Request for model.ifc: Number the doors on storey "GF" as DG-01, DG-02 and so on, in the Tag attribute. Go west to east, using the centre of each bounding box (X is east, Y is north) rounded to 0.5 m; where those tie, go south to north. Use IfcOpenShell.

First a look at what the model holds.

```python
import ifcopenshell
import ifcopenshell.util.element
import ifcopenshell.util.placement

model = ifcopenshell.open("model.ifc")
print(model.schema)
storey = next(s for s in model.by_type("IfcBuildingStorey") if s.Name == "GF")
doors = [e for e in ifcopenshell.util.element.get_decomposition(storey) if e.is_a("IfcDoor")]
for e in sorted(doors, key=lambda e: e.id()):
    origin = ifcopenshell.util.placement.get_local_placement(e.ObjectPlacement)[:3, 3]
    print(e.id(), e.Tag, e.Name, origin.round(2) + 0.0, sep=" | ")
```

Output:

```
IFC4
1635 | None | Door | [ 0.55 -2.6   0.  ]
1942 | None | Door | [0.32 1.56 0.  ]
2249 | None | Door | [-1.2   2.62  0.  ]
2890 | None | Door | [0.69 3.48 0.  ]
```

```python
import ifcopenshell
import ifcopenshell.geom
import ifcopenshell.util.element
import ifcopenshell.util.shape

model = ifcopenshell.open("model.ifc")
settings = ifcopenshell.geom.settings()
settings.set("use-world-coords", True)


def centre(element):
    shape = ifcopenshell.geom.create_shape(settings, element)
    return ifcopenshell.util.shape.get_bbox_centroid(shape.geometry)


storey = next(s for s in model.by_type("IfcBuildingStorey") if s.Name == "GF")
doors = [e for e in ifcopenshell.util.element.get_decomposition(storey) if e.is_a("IfcDoor")]

# Insertion points can sit at a corner or the storey origin, so sort by the geometry (in metres).
centres = {e: centre(e) for e in doors}
doors.sort(key=lambda e: (round(centres[e][0] / 0.5), centres[e][1]))

for i, e in enumerate(doors, start=1):
    number = f"DG-{i:02d}"
    e.Tag = number
    print(e.id(), number)

model.write("model_v2.ifc")
```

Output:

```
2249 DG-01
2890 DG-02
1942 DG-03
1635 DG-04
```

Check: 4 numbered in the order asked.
